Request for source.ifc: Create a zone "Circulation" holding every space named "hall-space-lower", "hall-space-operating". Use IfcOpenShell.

First a look at what the model holds.

```python
import ifcopenshell

model = ifcopenshell.open("source.ifc")
print(model.schema)
seen = {}
for space in model.by_type("IfcSpace"):
    seen[space.LongName] = seen.get(space.LongName, 0) + 1
for name, count in sorted(seen.items(), key=str):
    print(count, "x", name)
print("zones:", [z.Name for z in model.by_type("IfcZone")][:20])
```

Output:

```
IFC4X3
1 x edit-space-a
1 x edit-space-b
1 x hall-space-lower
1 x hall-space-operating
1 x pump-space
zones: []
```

```python
import ifcopenshell
import ifcopenshell.api.group
import ifcopenshell.api.root

model = ifcopenshell.open("source.ifc")

names = {"hall-space-lower", "hall-space-operating"}
spaces = [s for s in model.by_type("IfcSpace") if s.LongName in names]

zone = ifcopenshell.api.root.create_entity(model, ifc_class="IfcZone", name="Circulation")
ifcopenshell.api.group.assign_group(model, products=spaces, group=zone)
print(len(spaces), "spaces in", zone.Name)

model.write("source_edited.ifc")
```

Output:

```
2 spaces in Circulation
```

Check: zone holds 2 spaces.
